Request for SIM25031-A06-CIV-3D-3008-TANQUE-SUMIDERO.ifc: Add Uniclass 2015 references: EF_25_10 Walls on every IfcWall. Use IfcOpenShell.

First a look at what the model holds.

```python
import ifcopenshell

model = ifcopenshell.open("SIM25031-A06-CIV-3D-3008-TANQUE-SUMIDERO.ifc")
print(model.schema)
print("classifications:", [c.Name for c in model.by_type("IfcClassification")])
for ifc_class in ("IfcDoor", "IfcRoof", "IfcStair", "IfcWall", "IfcWindow"):
    print(ifc_class, len(model.by_type(ifc_class)))
```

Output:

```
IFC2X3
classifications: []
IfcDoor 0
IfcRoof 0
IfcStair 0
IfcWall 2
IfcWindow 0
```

```python
import ifcopenshell
import ifcopenshell.api.classification

model = ifcopenshell.open("SIM25031-A06-CIV-3D-3008-TANQUE-SUMIDERO.ifc")

# IFC2X3 requires Source and Edition and has no link from the project to the system.
system = model.create_entity("IfcClassification", Source="NBS", Edition="2015", Name="Uniclass 2015")

codes = {
    "IfcWall": ("EF_25_10", "Walls"),
}
for ifc_class, (code, name) in codes.items():
    products = model.by_type(ifc_class)
    ifcopenshell.api.classification.add_reference(
        model, products=products, classification=system, identification=code, name=name
    )
    print(code, len(products))

model.write("SIM25031-A06-CIV-3D-3008-TANQUE-SUMIDERO_updated.ifc")
```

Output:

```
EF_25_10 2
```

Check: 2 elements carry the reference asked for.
